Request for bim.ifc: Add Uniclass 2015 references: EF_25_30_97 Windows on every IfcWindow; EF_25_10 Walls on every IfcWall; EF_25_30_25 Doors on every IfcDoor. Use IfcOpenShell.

First a look at what the model holds.

```python
import ifcopenshell

model = ifcopenshell.open("bim.ifc")
print(model.schema)
print("classifications:", [c.Name for c in model.by_type("IfcClassification")])
for ifc_class in ("IfcDoor", "IfcRoof", "IfcStair", "IfcWall", "IfcWindow"):
    print(ifc_class, len(model.by_type(ifc_class)))
```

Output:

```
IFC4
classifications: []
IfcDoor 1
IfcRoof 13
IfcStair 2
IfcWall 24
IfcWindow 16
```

```python
import ifcopenshell
import ifcopenshell.api.classification

model = ifcopenshell.open("bim.ifc")

system = ifcopenshell.api.classification.add_classification(model, classification="Uniclass 2015")

codes = {
    "IfcWindow": ("EF_25_30_97", "Windows"),
    "IfcWall": ("EF_25_10", "Walls"),
    "IfcDoor": ("EF_25_30_25", "Doors"),
}
for ifc_class, (code, name) in codes.items():
    products = model.by_type(ifc_class)
    ifcopenshell.api.classification.add_reference(
        model, products=products, classification=system, identification=code, name=name
    )
    print(code, len(products))

model.write("bim-out.ifc")
```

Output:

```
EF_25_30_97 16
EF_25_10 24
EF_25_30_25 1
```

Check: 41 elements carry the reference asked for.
